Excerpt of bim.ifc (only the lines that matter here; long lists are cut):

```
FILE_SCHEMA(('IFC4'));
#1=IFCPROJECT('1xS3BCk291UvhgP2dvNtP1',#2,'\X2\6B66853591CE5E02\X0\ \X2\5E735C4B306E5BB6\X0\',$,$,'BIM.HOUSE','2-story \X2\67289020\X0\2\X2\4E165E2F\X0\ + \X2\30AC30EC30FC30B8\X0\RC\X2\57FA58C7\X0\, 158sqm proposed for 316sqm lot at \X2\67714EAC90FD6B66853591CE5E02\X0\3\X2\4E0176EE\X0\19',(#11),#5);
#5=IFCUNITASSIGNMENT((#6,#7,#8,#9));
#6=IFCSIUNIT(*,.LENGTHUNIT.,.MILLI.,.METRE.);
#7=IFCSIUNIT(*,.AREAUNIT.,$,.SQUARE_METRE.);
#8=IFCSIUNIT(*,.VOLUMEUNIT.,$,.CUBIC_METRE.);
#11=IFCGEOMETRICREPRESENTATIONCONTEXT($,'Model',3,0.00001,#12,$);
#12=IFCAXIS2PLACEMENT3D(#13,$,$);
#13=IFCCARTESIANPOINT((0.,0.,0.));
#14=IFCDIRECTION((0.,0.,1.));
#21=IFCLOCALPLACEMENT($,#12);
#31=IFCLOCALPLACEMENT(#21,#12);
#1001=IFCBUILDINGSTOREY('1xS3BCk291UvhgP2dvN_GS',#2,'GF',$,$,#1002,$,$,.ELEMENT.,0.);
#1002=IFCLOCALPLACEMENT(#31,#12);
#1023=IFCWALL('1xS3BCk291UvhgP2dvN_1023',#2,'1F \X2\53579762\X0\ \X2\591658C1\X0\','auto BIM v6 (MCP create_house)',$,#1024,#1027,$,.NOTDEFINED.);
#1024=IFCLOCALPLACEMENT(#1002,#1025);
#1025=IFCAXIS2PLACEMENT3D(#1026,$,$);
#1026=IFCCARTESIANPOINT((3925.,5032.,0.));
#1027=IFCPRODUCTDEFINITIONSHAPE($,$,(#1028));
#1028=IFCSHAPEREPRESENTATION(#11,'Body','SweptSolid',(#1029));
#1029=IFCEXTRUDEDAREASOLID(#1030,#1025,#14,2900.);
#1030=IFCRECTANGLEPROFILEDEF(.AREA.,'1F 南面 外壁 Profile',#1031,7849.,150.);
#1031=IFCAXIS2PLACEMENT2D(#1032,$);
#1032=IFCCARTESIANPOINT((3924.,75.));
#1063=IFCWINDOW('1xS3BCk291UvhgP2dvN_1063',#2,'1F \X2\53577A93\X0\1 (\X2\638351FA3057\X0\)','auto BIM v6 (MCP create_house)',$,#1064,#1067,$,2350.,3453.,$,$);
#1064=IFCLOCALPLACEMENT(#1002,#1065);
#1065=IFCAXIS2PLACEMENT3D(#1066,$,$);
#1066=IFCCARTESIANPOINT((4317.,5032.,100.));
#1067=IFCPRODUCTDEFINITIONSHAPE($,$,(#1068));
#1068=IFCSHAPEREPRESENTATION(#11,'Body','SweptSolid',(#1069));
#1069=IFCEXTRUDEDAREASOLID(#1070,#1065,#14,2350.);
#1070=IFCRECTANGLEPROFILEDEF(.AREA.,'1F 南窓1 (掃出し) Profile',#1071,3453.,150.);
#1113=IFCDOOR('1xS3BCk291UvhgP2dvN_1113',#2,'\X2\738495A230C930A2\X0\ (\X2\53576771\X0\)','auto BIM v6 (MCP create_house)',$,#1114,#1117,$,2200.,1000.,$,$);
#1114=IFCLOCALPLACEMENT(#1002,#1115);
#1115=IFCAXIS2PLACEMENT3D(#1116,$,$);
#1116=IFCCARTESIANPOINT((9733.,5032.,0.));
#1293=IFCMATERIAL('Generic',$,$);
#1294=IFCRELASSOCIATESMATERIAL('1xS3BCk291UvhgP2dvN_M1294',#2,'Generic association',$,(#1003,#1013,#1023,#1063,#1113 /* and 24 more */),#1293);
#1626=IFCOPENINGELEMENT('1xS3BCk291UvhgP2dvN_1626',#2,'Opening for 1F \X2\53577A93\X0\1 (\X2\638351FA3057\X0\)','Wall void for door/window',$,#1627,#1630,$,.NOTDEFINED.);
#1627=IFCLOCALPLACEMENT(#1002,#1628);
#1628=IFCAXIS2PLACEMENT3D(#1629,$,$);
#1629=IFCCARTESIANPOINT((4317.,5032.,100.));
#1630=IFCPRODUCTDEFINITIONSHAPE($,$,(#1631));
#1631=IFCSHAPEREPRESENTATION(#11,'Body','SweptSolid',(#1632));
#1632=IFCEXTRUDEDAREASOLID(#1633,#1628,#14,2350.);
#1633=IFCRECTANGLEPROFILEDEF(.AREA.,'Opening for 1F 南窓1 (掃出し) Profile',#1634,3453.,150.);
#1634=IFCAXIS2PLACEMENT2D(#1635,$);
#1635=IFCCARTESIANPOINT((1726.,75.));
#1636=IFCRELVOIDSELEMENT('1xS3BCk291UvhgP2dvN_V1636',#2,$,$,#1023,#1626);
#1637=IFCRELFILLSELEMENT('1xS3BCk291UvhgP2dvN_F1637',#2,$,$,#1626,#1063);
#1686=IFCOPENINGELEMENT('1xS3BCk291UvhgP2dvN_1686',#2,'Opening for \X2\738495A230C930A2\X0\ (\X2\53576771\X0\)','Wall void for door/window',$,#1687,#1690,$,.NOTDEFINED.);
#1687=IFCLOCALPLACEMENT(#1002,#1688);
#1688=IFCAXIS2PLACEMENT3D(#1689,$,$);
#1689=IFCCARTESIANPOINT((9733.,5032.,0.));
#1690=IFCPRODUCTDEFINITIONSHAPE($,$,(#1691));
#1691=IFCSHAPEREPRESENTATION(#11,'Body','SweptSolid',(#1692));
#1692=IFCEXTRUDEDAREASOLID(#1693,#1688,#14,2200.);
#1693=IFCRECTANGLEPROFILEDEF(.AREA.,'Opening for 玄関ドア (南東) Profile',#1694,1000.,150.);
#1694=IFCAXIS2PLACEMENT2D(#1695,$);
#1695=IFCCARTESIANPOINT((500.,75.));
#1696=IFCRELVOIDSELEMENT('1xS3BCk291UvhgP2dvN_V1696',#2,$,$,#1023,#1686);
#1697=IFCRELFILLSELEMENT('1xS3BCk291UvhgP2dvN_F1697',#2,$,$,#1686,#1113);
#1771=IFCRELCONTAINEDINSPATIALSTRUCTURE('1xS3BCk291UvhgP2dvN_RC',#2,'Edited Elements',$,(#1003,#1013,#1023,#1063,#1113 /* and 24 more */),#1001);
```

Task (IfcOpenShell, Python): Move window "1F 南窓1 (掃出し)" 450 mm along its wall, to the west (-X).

```python
import ifcopenshell
import ifcopenshell.api.geometry
import ifcopenshell.util.placement
import ifcopenshell.util.unit

model = ifcopenshell.open("bim.ifc")
unit_scale = ifcopenshell.util.unit.calculate_unit_scale(model)

window = model.by_id(1063)
opening = window.FillsVoids[0].RelatingOpeningElement
wall = opening.VoidsElements[0].RelatingBuildingElement

wall_matrix = ifcopenshell.util.placement.get_local_placement(wall.ObjectPlacement)
shift = wall_matrix[:3, 0] * -0.45 / unit_scale
before = ifcopenshell.util.placement.get_local_placement(window.ObjectPlacement)[:3, 3].copy()

# The window is not placed relative to its opening, so move both.
for product in (opening, window):
    matrix = ifcopenshell.util.placement.get_local_placement(product.ObjectPlacement)
    matrix[:3, 3] += shift
    ifcopenshell.api.geometry.edit_object_placement(model, product=product, matrix=matrix, is_si=False)

after = ifcopenshell.util.placement.get_local_placement(window.ObjectPlacement)[:3, 3]
print("window moved by", (after - before).round(3) + 0.0)

model.write("bim_rev.ifc")
```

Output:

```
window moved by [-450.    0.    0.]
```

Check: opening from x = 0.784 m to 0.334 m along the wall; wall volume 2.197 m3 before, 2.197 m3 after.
